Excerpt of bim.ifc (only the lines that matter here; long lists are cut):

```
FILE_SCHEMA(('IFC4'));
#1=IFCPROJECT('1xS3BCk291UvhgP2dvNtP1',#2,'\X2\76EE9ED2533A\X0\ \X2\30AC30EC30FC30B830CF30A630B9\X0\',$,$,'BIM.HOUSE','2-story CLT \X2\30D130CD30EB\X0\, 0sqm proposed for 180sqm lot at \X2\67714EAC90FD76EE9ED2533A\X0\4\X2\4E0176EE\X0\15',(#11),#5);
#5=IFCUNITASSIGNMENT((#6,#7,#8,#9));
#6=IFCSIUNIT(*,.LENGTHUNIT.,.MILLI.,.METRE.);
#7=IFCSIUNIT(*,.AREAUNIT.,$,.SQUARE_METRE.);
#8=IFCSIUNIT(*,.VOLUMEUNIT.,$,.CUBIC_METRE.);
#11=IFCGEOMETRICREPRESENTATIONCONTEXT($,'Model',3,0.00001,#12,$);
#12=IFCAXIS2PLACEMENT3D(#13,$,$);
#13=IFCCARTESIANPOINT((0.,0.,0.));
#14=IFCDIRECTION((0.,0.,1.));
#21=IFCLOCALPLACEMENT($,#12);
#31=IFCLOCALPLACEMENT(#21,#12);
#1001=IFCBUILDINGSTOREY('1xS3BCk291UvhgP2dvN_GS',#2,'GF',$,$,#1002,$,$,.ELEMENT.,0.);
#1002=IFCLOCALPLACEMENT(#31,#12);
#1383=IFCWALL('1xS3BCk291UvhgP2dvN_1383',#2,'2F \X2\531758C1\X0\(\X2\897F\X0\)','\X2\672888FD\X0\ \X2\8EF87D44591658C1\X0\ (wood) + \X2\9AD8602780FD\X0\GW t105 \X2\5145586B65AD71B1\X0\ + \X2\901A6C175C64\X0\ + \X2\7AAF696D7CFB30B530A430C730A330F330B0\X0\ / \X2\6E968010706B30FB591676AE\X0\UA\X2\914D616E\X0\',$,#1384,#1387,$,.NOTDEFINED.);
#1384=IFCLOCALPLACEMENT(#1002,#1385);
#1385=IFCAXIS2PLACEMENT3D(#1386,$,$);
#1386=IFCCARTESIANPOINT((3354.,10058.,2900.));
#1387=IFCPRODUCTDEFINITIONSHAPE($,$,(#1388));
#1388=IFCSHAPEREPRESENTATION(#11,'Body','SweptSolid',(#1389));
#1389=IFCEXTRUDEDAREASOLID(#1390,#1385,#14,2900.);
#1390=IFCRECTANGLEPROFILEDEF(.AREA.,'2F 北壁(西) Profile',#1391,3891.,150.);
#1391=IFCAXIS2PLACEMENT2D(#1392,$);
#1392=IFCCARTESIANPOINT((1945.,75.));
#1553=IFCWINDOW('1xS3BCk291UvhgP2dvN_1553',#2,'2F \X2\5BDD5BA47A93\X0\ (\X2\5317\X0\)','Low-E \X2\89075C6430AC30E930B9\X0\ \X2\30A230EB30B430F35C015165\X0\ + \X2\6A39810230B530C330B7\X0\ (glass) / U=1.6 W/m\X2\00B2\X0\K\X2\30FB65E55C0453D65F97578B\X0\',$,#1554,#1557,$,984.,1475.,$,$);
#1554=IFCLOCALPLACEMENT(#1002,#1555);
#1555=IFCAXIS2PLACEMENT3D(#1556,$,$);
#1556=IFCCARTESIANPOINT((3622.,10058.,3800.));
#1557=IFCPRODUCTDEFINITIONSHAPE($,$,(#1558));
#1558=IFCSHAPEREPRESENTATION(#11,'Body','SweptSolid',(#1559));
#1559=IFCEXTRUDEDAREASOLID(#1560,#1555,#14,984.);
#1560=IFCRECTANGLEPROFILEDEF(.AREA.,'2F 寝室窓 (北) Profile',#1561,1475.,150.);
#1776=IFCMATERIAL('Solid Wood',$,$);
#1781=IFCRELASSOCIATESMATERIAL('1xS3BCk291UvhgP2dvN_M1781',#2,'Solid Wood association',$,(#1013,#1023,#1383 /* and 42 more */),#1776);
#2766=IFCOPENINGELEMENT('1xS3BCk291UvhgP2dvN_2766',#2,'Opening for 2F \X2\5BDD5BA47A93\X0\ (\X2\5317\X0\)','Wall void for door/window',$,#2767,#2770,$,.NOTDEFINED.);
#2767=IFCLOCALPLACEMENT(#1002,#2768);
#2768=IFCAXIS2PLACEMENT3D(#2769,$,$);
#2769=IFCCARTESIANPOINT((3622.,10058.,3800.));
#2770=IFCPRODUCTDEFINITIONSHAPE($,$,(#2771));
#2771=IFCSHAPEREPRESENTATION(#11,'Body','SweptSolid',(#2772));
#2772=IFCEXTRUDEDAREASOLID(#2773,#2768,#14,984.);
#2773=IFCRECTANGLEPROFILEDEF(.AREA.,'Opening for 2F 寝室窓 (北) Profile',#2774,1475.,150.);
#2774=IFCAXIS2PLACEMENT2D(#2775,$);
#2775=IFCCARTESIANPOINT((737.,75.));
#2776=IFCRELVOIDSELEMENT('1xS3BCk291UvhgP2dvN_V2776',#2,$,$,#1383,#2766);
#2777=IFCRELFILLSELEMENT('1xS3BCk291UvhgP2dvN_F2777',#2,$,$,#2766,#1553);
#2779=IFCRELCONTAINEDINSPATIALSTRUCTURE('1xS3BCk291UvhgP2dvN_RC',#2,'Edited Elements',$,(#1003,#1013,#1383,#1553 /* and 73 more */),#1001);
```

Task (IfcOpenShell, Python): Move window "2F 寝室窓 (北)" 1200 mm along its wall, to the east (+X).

```python
import ifcopenshell
import ifcopenshell.api.geometry
import ifcopenshell.util.placement

model = ifcopenshell.open("bim.ifc")

window = model.by_guid("1xS3BCk291UvhgP2dvN_1553")
opening = window.FillsVoids[0].RelatingOpeningElement
wall = opening.VoidsElements[0].RelatingBuildingElement

wall_matrix = ifcopenshell.util.placement.get_local_placement(wall.ObjectPlacement)
shift = wall_matrix[:3, 0] * 1200.0
before = ifcopenshell.util.placement.get_local_placement(window.ObjectPlacement)[:3, 3].copy()

# The window is not placed relative to its opening, so move both.
for product in (opening, window):
    matrix = ifcopenshell.util.placement.get_local_placement(product.ObjectPlacement)
    matrix[:3, 3] += shift
    ifcopenshell.api.geometry.edit_object_placement(model, product=product, matrix=matrix, is_si=False)

after = ifcopenshell.util.placement.get_local_placement(window.ObjectPlacement)[:3, 3]
print("window moved by", (after - before).round(3) + 0.0)

model.write("bim_rev.ifc")
```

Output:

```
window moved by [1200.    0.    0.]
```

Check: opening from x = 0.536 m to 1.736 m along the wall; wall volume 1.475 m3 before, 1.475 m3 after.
